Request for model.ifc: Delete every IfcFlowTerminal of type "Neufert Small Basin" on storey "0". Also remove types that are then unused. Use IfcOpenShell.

First a look at what the model holds.

```python
import ifcopenshell
import ifcopenshell.util.element

model = ifcopenshell.open("model.ifc")
print(model.schema)
storey = next(s for s in model.by_type("IfcBuildingStorey") if s.Name == "0")
terminals = [e for e in ifcopenshell.util.element.get_decomposition(storey) if e.is_a("IfcFlowTerminal")]
seen = {}
for e in terminals:
    element_type = ifcopenshell.util.element.get_type(e)
    name = element_type.Name if element_type not in (None, e) else None
    seen[name] = seen.get(name, 0) + 1
for name, count in sorted(seen.items(), key=str):
    print(count, "x", name)
```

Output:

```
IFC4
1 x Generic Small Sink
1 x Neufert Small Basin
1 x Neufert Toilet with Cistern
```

```python
import ifcopenshell
import ifcopenshell.api.root
import ifcopenshell.util.element

model = ifcopenshell.open("model.ifc")

storey = next(s for s in model.by_type("IfcBuildingStorey") if s.Name == "0")
terminals = [e for e in ifcopenshell.util.element.get_decomposition(storey) if e.is_a("IfcFlowTerminal")]
targets = [e for e in terminals if (t := ifcopenshell.util.element.get_type(e)) not in (None, e) and t.Name == "Neufert Small Basin"]
types = {ifcopenshell.util.element.get_type(e) for e in targets} - {None, *targets}

for e in targets:
    ifcopenshell.api.root.remove_product(model, product=e)
print(len(targets), "removed")

unused = [t for t in types if not ifcopenshell.util.element.get_types(t)]
for t in unused:
    ifcopenshell.api.root.remove_product(model, product=t)
print(len(unused), "unused types removed")

model.write("model_v2.ifc")
```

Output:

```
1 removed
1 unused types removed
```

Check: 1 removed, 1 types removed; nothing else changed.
